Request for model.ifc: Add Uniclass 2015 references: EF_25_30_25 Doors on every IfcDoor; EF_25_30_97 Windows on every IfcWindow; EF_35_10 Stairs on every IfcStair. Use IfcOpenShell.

First a look at what the model holds.

```python
import ifcopenshell

model = ifcopenshell.open("model.ifc")
print(model.schema)
print("classifications:", [c.Name for c in model.by_type("IfcClassification")])
for ifc_class in ("IfcDoor", "IfcRoof", "IfcStair", "IfcWall", "IfcWindow"):
    print(ifc_class, len(model.by_type(ifc_class)))
```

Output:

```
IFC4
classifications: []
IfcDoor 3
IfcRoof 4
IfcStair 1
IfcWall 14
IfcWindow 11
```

```python
import ifcopenshell
import ifcopenshell.api.classification

model = ifcopenshell.open("model.ifc")

system = ifcopenshell.api.classification.add_classification(model, classification="Uniclass 2015")

codes = {
    "IfcDoor": ("EF_25_30_25", "Doors"),
    "IfcWindow": ("EF_25_30_97", "Windows"),
    "IfcStair": ("EF_35_10", "Stairs"),
}
for ifc_class, (code, name) in codes.items():
    products = model.by_type(ifc_class)
    ifcopenshell.api.classification.add_reference(
        model, products=products, classification=system, identification=code, name=name
    )
    print(code, len(products))

model.write("model_rev.ifc")
```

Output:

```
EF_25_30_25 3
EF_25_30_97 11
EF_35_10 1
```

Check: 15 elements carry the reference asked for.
